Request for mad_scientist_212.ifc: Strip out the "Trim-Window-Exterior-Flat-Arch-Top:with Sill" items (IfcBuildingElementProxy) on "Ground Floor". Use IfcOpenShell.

First a look at what the model holds.

```python
import ifcopenshell
import ifcopenshell.util.element

model = ifcopenshell.open("mad_scientist_212.ifc")
print(model.schema)
storey = next(s for s in model.by_type("IfcBuildingStorey") if s.Name == "Ground Floor")
proxies = [e for e in ifcopenshell.util.element.get_decomposition(storey) if e.is_a("IfcBuildingElementProxy")]
seen = {}
for e in proxies:
    element_type = ifcopenshell.util.element.get_type(e)
    name = element_type.Name if element_type not in (None, e) else None
    seen[name] = seen.get(name, 0) + 1
for name, count in sorted(seen.items(), key=str):
    print(count, "x", name)
```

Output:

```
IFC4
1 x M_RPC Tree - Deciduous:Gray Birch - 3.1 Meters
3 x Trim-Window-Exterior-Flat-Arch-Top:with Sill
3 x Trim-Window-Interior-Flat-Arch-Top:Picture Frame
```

```python
import ifcopenshell
import ifcopenshell.api.root
import ifcopenshell.util.element

model = ifcopenshell.open("mad_scientist_212.ifc")

storey = next(s for s in model.by_type("IfcBuildingStorey") if s.Name == "Ground Floor")
proxies = [e for e in ifcopenshell.util.element.get_decomposition(storey) if e.is_a("IfcBuildingElementProxy")]
targets = [e for e in proxies if (t := ifcopenshell.util.element.get_type(e)) not in (None, e) and t.Name == "Trim-Window-Exterior-Flat-Arch-Top:with Sill"]

for e in targets:
    ifcopenshell.api.root.remove_product(model, product=e)
print(len(targets), "removed")

model.write("mad_scientist_212_edited.ifc")
```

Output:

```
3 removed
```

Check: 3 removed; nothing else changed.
